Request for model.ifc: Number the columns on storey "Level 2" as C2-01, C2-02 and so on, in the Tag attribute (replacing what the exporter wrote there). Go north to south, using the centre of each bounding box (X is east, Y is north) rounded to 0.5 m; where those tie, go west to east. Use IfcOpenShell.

First a look at what the model holds.

```python
import ifcopenshell
import ifcopenshell.util.element
import ifcopenshell.util.placement

model = ifcopenshell.open("model.ifc")
print(model.schema)
storey = next(s for s in model.by_type("IfcBuildingStorey") if s.Name == "Level 2")
columns = [e for e in ifcopenshell.util.element.get_decomposition(storey) if e.is_a("IfcColumn")]
for e in sorted(columns, key=lambda e: e.id()):
    origin = ifcopenshell.util.placement.get_local_placement(e.ObjectPlacement)[:3, 3]
    print(e.id(), e.Tag, e.Name, origin.round(2) + 0.0, sep=" | ")
```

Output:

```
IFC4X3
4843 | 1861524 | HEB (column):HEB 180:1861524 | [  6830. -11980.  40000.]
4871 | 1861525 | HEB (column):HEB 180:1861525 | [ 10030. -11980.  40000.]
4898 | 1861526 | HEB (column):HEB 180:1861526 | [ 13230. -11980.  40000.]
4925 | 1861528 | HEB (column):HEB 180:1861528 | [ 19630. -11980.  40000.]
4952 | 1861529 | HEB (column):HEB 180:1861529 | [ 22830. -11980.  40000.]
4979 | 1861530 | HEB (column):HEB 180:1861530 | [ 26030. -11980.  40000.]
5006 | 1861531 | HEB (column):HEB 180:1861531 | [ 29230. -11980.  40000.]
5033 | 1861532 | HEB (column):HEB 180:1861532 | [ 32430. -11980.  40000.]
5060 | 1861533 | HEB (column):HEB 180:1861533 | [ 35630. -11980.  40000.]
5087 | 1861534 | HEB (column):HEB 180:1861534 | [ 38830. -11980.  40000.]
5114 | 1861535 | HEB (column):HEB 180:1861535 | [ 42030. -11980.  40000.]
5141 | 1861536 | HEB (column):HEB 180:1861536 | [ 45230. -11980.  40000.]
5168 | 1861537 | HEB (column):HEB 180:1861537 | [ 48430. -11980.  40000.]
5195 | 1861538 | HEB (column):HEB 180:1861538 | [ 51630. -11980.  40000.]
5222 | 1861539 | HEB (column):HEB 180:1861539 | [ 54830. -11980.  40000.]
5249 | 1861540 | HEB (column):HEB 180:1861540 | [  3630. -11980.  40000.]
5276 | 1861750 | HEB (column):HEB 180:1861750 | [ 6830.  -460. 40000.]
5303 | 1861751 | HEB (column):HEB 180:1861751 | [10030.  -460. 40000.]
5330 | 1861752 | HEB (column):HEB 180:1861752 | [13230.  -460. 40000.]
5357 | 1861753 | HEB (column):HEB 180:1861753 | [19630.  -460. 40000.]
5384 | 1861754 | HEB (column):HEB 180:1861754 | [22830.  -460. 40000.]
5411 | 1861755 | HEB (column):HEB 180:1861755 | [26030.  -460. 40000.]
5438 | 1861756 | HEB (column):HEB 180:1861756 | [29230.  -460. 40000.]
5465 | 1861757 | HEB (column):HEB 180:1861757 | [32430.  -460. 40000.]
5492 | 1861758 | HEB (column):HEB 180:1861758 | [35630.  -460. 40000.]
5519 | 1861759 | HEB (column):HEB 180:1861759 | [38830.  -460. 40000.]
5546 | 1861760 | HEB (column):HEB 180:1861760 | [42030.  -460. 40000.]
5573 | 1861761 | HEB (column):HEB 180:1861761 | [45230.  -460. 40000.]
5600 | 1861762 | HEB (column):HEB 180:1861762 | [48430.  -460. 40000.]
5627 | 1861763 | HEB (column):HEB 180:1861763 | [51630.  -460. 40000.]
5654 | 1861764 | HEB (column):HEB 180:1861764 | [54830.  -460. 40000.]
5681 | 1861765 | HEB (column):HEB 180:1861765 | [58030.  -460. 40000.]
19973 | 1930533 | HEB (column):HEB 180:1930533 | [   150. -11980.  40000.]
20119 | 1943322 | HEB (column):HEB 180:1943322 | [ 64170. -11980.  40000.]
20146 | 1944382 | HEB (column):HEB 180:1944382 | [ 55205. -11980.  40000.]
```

```python
import ifcopenshell
import ifcopenshell.geom
import ifcopenshell.util.element
import ifcopenshell.util.shape

model = ifcopenshell.open("model.ifc")
settings = ifcopenshell.geom.settings()
settings.set("use-world-coords", True)


def centre(element):
    shape = ifcopenshell.geom.create_shape(settings, element)
    return ifcopenshell.util.shape.get_bbox_centroid(shape.geometry)


storey = next(s for s in model.by_type("IfcBuildingStorey") if s.Name == "Level 2")
columns = [e for e in ifcopenshell.util.element.get_decomposition(storey) if e.is_a("IfcColumn")]

# Insertion points can sit at a corner or the storey origin, so sort by the geometry (in metres).
centres = {e: centre(e) for e in columns}
columns.sort(key=lambda e: (-round(centres[e][1] / 0.5), centres[e][0]))

for i, e in enumerate(columns, start=1):
    number = f"C2-{i:02d}"
    e.Tag = number
    print(e.id(), number)

model.write("model-out.ifc")
```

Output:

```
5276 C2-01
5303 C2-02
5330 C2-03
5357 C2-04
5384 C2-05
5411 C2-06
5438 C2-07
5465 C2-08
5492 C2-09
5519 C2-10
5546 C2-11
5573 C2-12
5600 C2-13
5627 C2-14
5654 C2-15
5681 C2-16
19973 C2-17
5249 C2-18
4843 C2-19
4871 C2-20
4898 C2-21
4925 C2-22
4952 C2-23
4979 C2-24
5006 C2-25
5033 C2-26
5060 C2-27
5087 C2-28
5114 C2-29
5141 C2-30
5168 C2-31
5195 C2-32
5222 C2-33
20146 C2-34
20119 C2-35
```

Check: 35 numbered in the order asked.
